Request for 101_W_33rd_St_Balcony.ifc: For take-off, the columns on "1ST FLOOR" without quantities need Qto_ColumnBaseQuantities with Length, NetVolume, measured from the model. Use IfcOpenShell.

First a look at what the model holds.

```python
import ifcopenshell
import ifcopenshell.util.element
import ifcopenshell.util.unit

model = ifcopenshell.open("101_W_33rd_St_Balcony.ifc")
print(model.schema)
for unit_type in ("LENGTHUNIT", "AREAUNIT", "VOLUMEUNIT"):
    print(unit_type, ifcopenshell.util.unit.calculate_unit_scale(model, unit_type))
storey = next(s for s in model.by_type("IfcBuildingStorey") if s.Name == "1ST FLOOR")
columns = [e for e in ifcopenshell.util.element.get_decomposition(storey) if e.is_a("IfcColumn")]
for e in sorted(columns, key=lambda e: e.id()):
    print(e.id(), e.is_a(), e.Name, list(ifcopenshell.util.element.get_psets(e, qtos_only=True)), sep=" | ")
```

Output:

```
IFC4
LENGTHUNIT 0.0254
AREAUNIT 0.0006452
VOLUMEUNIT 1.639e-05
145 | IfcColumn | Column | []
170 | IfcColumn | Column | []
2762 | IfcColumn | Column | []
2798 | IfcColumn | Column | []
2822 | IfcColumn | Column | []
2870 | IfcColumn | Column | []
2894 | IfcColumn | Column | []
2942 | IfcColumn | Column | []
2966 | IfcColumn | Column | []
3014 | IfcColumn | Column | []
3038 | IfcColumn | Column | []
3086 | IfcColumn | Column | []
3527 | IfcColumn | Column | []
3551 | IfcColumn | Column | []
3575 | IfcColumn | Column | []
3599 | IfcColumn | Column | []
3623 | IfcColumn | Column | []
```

```python
import ifcopenshell
import ifcopenshell.api.pset
import ifcopenshell.geom
import ifcopenshell.util.element
import ifcopenshell.util.shape
import ifcopenshell.util.unit

model = ifcopenshell.open("101_W_33rd_St_Balcony.ifc")
unit_scale = ifcopenshell.util.unit.calculate_unit_scale(model)
volume_scale = ifcopenshell.util.unit.calculate_unit_scale(model, "VOLUMEUNIT")
settings = ifcopenshell.geom.settings()

storey = next(s for s in model.by_type("IfcBuildingStorey") if s.Name == "1ST FLOOR")
columns = [e for e in ifcopenshell.util.element.get_decomposition(storey) if e.is_a("IfcColumn")]

for e in sorted(columns, key=lambda e: e.id()):
    if ifcopenshell.util.element.get_psets(e, qtos_only=True, should_inherit=False):
        continue
    # Geometry comes back in metres, in the element's own axes.
    shape = ifcopenshell.geom.create_shape(settings, e)
    values = {
        "Length": ifcopenshell.util.shape.get_z(shape.geometry) / unit_scale,
        "NetVolume": ifcopenshell.util.shape.get_volume(shape.geometry) / volume_scale,
    }
    qto = ifcopenshell.api.pset.add_qto(model, product=e, name="Qto_ColumnBaseQuantities")
    ifcopenshell.api.pset.edit_qto(model, qto=qto, properties=values)
    print(e.id(), {k: round(v, 3) for k, v in values.items()})

model.write("101_W_33rd_St_Balcony_updated.ifc")
```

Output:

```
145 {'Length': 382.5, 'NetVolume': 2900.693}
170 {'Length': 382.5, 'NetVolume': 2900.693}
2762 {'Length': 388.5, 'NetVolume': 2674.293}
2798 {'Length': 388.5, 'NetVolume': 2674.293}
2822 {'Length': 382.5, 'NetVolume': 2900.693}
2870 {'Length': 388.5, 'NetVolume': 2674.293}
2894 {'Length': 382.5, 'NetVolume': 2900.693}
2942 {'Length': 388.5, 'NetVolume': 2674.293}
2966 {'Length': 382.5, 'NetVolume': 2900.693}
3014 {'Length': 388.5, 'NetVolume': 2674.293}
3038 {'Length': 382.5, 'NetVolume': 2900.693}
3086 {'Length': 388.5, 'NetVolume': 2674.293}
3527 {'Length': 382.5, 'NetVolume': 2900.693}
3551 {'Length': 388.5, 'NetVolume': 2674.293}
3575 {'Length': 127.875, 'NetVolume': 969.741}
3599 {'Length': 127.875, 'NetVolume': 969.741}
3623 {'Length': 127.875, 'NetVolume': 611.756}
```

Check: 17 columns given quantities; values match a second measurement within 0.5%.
